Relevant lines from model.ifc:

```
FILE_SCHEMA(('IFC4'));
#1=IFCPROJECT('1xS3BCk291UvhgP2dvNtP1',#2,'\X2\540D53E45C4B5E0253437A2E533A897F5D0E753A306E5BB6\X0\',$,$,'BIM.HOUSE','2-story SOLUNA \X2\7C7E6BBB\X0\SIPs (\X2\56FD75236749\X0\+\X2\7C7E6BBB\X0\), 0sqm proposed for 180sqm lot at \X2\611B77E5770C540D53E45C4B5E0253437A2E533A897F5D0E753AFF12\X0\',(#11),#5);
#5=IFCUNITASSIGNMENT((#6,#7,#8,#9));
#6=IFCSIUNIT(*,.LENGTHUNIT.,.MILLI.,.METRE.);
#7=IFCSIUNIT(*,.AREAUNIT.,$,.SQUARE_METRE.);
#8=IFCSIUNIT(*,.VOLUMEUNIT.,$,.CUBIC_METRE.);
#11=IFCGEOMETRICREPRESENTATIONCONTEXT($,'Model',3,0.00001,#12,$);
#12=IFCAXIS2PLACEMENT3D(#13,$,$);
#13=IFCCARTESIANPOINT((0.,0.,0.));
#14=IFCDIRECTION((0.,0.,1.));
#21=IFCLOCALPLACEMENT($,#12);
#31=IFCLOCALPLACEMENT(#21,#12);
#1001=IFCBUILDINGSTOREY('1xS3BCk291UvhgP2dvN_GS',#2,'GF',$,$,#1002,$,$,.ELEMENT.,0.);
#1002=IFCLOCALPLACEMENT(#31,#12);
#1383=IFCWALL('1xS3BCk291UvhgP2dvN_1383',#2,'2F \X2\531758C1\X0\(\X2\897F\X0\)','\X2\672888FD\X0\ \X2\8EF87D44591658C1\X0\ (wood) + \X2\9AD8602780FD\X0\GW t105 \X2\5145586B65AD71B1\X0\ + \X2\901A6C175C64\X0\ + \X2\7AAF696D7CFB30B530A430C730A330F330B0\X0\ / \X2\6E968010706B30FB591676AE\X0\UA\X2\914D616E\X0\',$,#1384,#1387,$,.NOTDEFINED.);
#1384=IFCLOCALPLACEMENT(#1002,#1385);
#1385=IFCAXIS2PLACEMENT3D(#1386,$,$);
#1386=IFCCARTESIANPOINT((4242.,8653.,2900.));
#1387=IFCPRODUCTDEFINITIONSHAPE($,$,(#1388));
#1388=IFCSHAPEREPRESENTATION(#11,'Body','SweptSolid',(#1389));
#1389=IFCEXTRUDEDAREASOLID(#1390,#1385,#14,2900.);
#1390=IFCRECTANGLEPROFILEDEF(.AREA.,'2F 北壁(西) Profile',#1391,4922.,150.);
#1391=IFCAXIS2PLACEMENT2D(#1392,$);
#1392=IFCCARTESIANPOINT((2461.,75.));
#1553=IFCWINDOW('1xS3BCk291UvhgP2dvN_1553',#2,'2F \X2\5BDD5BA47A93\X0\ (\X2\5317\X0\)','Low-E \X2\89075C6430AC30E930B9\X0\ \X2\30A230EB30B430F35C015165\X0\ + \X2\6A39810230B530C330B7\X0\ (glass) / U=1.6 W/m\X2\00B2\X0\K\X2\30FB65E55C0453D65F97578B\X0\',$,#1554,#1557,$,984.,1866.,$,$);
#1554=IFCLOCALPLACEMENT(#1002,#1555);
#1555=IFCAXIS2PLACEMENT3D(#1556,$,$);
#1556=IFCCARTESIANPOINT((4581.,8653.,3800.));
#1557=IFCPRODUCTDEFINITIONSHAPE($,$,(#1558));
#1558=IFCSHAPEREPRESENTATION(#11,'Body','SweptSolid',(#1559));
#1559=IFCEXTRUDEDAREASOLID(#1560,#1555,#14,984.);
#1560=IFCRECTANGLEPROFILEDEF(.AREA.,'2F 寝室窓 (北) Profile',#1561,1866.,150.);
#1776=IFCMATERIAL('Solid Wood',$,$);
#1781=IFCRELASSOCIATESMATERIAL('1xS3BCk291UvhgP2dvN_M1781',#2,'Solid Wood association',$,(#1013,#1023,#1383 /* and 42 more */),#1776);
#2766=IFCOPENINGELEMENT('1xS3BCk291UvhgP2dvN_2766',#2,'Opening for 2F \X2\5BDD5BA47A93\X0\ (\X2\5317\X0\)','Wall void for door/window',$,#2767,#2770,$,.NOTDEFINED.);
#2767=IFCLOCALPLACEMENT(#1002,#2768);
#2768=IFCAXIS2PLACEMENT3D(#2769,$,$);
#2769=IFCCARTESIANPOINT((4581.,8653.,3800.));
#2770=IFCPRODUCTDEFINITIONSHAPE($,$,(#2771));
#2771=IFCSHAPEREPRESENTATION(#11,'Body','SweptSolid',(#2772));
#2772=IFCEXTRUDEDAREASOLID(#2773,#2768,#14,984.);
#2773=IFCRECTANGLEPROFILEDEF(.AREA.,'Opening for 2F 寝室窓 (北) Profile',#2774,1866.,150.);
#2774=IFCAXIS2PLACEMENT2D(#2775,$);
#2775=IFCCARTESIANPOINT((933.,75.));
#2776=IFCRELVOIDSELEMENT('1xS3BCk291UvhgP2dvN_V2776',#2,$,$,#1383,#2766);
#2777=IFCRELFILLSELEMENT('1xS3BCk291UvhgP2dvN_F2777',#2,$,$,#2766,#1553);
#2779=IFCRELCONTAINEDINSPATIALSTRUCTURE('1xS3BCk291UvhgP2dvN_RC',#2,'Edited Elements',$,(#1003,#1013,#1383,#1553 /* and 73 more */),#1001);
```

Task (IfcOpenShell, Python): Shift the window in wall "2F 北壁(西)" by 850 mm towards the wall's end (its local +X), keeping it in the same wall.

```python
import ifcopenshell
import ifcopenshell.api.geometry
import ifcopenshell.util.placement

model = ifcopenshell.open("model.ifc")

window = model.by_guid("1xS3BCk291UvhgP2dvN_1553")
opening = window.FillsVoids[0].RelatingOpeningElement
wall = opening.VoidsElements[0].RelatingBuildingElement

wall_matrix = ifcopenshell.util.placement.get_local_placement(wall.ObjectPlacement)
shift = wall_matrix[:3, 0] * 850.0
before = ifcopenshell.util.placement.get_local_placement(window.ObjectPlacement)[:3, 3].copy()

# The window is not placed relative to its opening, so move both.
for product in (opening, window):
    matrix = ifcopenshell.util.placement.get_local_placement(product.ObjectPlacement)
    matrix[:3, 3] += shift
    ifcopenshell.api.geometry.edit_object_placement(model, product=product, matrix=matrix, is_si=False)

after = ifcopenshell.util.placement.get_local_placement(window.ObjectPlacement)[:3, 3]
print("window moved by", (after - before).round(3) + 0.0)

model.write("model_rev.ifc")
```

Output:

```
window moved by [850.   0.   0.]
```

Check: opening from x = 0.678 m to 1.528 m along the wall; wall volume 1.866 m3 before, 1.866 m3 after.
